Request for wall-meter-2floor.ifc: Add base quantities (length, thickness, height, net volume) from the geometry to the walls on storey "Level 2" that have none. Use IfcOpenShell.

First a look at what the model holds.

```python
import ifcopenshell
import ifcopenshell.util.element
import ifcopenshell.util.unit

model = ifcopenshell.open("wall-meter-2floor.ifc")
print(model.schema)
for unit_type in ("LENGTHUNIT", "AREAUNIT", "VOLUMEUNIT"):
    print(unit_type, ifcopenshell.util.unit.calculate_unit_scale(model, unit_type))
storey = next(s for s in model.by_type("IfcBuildingStorey") if s.Name == "Level 2")
walls = [e for e in ifcopenshell.util.element.get_decomposition(storey) if e.is_a("IfcWall")]
for e in sorted(walls, key=lambda e: e.id()):
    print(e.id(), e.is_a(), e.Name, list(ifcopenshell.util.element.get_psets(e, qtos_only=True)), sep=" | ")
```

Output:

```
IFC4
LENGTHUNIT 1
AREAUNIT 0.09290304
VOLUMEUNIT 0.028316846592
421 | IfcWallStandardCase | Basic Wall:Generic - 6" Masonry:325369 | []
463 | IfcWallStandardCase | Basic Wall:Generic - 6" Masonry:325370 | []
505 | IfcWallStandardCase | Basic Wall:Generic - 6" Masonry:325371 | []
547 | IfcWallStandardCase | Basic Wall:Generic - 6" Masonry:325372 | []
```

```python
import ifcopenshell
import ifcopenshell.api.pset
import ifcopenshell.geom
import ifcopenshell.util.element
import ifcopenshell.util.shape
import ifcopenshell.util.unit

model = ifcopenshell.open("wall-meter-2floor.ifc")
unit_scale = ifcopenshell.util.unit.calculate_unit_scale(model)
volume_scale = ifcopenshell.util.unit.calculate_unit_scale(model, "VOLUMEUNIT")
settings = ifcopenshell.geom.settings()

storey = next(s for s in model.by_type("IfcBuildingStorey") if s.Name == "Level 2")
walls = [e for e in ifcopenshell.util.element.get_decomposition(storey) if e.is_a("IfcWall")]

for e in sorted(walls, key=lambda e: e.id()):
    if ifcopenshell.util.element.get_psets(e, qtos_only=True, should_inherit=False):
        continue
    # Geometry comes back in metres, in the element's own axes.
    shape = ifcopenshell.geom.create_shape(settings, e)
    values = {
        "Length": ifcopenshell.util.shape.get_x(shape.geometry) / unit_scale,
        "Width": ifcopenshell.util.shape.get_y(shape.geometry) / unit_scale,
        "Height": ifcopenshell.util.shape.get_z(shape.geometry) / unit_scale,
        "NetVolume": ifcopenshell.util.shape.get_volume(shape.geometry) / volume_scale,
    }
    qto = ifcopenshell.api.pset.add_qto(model, product=e, name="Qto_WallBaseQuantities")
    ifcopenshell.api.pset.edit_qto(model, qto=qto, properties=values)
    print(e.id(), {k: round(v, 3) for k, v in values.items()})

model.write("wall-meter-2floor_rev.ifc")
```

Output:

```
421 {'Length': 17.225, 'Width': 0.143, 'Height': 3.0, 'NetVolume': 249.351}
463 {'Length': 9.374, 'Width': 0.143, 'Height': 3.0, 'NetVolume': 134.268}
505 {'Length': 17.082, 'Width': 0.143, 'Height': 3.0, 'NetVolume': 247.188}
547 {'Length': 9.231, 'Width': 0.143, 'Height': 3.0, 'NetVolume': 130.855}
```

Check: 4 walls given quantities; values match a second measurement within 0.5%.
